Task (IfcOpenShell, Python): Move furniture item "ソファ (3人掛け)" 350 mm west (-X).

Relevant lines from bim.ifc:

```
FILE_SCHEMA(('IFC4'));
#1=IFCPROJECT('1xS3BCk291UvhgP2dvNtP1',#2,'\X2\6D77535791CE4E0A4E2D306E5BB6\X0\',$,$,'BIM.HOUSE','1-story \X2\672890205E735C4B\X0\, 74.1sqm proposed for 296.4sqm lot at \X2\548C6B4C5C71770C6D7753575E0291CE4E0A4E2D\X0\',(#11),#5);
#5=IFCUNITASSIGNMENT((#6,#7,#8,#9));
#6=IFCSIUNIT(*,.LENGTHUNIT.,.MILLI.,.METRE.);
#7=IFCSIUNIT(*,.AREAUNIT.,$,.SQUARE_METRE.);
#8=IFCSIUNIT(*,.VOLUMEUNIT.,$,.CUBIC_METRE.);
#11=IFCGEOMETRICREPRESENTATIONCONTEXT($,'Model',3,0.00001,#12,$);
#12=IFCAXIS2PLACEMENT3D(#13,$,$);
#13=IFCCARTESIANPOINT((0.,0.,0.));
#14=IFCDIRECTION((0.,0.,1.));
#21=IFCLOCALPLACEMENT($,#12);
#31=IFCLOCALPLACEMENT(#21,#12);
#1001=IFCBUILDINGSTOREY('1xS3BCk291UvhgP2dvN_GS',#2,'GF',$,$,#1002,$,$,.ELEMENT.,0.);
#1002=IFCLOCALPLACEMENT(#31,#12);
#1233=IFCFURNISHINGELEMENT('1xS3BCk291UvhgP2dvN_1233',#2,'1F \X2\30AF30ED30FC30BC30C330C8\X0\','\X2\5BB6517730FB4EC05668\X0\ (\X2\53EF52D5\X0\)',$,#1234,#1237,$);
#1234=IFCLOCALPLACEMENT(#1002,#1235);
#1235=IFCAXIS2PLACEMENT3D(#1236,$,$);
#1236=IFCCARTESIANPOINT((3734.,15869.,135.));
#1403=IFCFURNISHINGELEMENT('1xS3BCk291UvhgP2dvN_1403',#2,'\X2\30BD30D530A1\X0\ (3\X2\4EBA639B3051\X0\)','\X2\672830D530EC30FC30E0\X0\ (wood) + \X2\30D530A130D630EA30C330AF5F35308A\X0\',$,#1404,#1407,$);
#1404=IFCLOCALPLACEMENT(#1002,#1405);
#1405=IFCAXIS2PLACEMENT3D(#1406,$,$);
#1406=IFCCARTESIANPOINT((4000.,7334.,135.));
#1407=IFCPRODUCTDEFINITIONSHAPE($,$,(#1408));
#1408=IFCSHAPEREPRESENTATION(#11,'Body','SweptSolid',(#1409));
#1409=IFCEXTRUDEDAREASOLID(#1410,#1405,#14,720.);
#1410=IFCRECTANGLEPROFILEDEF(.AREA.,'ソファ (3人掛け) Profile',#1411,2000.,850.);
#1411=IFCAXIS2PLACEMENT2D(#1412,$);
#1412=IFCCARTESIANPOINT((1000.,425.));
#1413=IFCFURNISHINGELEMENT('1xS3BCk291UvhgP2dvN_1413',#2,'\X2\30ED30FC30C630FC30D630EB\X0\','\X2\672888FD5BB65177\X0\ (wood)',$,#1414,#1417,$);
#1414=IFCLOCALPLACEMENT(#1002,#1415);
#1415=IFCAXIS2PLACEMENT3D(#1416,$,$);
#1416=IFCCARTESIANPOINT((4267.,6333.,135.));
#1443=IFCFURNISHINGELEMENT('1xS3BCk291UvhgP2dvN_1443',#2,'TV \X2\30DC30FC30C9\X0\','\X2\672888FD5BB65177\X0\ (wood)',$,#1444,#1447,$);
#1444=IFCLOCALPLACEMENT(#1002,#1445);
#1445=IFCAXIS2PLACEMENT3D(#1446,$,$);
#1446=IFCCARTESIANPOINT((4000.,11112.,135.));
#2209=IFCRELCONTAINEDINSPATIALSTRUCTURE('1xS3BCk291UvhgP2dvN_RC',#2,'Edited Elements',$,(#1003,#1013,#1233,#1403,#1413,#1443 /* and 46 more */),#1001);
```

```python
import ifcopenshell
import ifcopenshell.api.geometry
import ifcopenshell.util.placement
import ifcopenshell.util.unit

model = ifcopenshell.open("bim.ifc")
unit_scale = ifcopenshell.util.unit.calculate_unit_scale(model)

item = model.by_guid("1xS3BCk291UvhgP2dvN_1403")
matrix = ifcopenshell.util.placement.get_local_placement(item.ObjectPlacement)
matrix[0, 3] -= 0.35 / unit_scale
ifcopenshell.api.geometry.edit_object_placement(model, product=item, matrix=matrix, is_si=False)

print(ifcopenshell.util.placement.get_local_placement(item.ObjectPlacement).round(3) + 0.0)

model.write("bim_edited.ifc")
```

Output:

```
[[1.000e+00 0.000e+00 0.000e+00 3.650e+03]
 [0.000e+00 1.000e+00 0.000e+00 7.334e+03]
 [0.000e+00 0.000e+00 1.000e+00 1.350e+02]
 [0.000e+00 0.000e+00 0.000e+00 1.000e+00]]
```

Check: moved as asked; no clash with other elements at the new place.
